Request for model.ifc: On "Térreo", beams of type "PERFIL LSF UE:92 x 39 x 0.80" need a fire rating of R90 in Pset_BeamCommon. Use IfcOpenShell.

First a look at what the model holds.

```python
import ifcopenshell
import ifcopenshell.util.element

model = ifcopenshell.open("model.ifc")
print(model.schema)
storey = next(s for s in model.by_type("IfcBuildingStorey") if s.Name == "Térreo")
beams = [e for e in ifcopenshell.util.element.get_decomposition(storey) if e.is_a("IfcBeam")]
seen = {}
for e in beams:
    element_type = ifcopenshell.util.element.get_type(e)
    key = (element_type.Name if element_type != e and element_type else None, ifcopenshell.util.element.get_pset(e, "Pset_BeamCommon", "FireRating"))
    seen[key] = seen.get(key, 0) + 1
for (name, value), count in sorted(seen.items(), key=str):
    print(count, "x", name, "|", value)
```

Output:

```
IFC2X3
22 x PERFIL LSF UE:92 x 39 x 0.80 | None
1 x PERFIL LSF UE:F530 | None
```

```python
import ifcopenshell
import ifcopenshell.api.pset
import ifcopenshell.util.element

model = ifcopenshell.open("model.ifc")

storey = next(s for s in model.by_type("IfcBuildingStorey") if s.Name == "Térreo")
beams = [e for e in ifcopenshell.util.element.get_decomposition(storey) if e.is_a("IfcBeam")]

count = 0
for e in beams:
    element_type = ifcopenshell.util.element.get_type(e)
    if element_type in (None, e) or element_type.Name != "PERFIL LSF UE:92 x 39 x 0.80":
        continue
    # add_pset returns the element's existing set when there is one.
    pset = ifcopenshell.api.pset.add_pset(model, product=e, name="Pset_BeamCommon")
    ifcopenshell.api.pset.edit_pset(model, pset=pset, properties={"FireRating": "R90"})
    count += 1

print(count, "beams updated")

model.write("model_edited.ifc")
```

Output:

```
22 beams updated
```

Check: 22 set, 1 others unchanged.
